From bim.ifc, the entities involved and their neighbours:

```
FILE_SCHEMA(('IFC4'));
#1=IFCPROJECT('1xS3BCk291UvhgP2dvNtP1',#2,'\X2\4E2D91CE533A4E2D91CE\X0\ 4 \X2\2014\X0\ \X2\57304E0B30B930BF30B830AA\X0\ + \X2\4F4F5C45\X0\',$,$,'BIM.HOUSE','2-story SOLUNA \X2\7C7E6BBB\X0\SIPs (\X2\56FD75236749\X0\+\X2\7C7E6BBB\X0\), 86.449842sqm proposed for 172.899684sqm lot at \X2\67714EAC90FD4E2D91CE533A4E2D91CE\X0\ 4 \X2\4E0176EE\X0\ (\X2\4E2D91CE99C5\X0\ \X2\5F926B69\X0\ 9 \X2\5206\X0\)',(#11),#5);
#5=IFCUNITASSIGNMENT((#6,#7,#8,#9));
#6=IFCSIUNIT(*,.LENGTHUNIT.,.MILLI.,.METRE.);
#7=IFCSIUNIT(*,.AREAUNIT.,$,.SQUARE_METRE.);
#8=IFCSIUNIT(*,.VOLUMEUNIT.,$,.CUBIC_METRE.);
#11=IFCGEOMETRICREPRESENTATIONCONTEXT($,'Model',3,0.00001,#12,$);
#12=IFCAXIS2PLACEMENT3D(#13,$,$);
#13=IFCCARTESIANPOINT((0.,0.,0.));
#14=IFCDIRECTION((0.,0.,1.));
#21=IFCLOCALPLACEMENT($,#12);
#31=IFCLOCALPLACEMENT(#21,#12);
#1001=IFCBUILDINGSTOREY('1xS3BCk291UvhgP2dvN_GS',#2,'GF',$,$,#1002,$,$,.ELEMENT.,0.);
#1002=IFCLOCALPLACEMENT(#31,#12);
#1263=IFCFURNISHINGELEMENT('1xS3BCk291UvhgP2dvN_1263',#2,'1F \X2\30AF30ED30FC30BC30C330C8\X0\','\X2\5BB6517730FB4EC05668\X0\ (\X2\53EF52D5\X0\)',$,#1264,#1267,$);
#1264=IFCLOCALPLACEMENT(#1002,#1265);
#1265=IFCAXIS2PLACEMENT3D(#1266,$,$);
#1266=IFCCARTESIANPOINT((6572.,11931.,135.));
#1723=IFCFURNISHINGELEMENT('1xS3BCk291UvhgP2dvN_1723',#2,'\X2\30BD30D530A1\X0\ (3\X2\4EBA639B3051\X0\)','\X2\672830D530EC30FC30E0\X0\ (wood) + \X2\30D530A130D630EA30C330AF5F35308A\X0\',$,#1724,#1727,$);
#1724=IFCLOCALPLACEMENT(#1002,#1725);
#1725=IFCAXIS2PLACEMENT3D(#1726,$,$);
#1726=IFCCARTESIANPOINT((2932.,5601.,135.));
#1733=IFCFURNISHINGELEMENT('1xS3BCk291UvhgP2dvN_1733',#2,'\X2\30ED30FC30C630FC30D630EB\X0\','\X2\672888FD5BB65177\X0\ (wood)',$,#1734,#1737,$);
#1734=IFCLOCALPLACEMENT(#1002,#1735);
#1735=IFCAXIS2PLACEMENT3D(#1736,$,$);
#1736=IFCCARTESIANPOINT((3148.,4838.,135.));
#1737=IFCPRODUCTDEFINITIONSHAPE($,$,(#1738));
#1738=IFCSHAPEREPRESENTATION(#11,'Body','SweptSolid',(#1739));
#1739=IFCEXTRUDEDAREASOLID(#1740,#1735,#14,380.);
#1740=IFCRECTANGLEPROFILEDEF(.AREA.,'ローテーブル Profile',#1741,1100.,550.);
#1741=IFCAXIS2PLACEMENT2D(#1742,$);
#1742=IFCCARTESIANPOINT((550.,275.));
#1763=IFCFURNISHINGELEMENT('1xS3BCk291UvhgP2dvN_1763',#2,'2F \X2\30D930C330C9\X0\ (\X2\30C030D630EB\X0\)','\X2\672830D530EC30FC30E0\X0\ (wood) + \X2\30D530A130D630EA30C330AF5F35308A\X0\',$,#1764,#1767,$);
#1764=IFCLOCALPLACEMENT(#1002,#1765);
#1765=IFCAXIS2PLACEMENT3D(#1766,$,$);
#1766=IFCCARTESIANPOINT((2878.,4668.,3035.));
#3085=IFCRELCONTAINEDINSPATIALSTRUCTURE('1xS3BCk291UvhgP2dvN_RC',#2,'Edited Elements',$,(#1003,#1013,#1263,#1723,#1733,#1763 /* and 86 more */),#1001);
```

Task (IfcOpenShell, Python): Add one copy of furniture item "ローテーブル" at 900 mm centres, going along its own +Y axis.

```python
import ifcopenshell
import ifcopenshell.api.geometry
import ifcopenshell.api.root
import ifcopenshell.util.element
import ifcopenshell.util.placement
import ifcopenshell.util.unit

model = ifcopenshell.open("bim.ifc")
unit_scale = ifcopenshell.util.unit.calculate_unit_scale(model)


def reuse_history(source, copy):
    """copy_class also copies each property set's owner history, people and application; keep the originals."""
    for rel in copy.IsDefinedBy:
        if rel.is_a("IfcRelDefinesByProperties") and (history := rel.RelatingPropertyDefinition.OwnerHistory):
            rel.RelatingPropertyDefinition.OwnerHistory = source.OwnerHistory
            ifcopenshell.util.element.remove_deep2(model, history)


source = model.by_guid("1xS3BCk291UvhgP2dvN_1733")
base = ifcopenshell.util.placement.get_local_placement(source.ObjectPlacement)
step = base[:3, 1] * 0.9 / unit_scale

for i in range(1, 2):
    copy = ifcopenshell.api.root.copy_class(model, product=source)
    copy.Representation = ifcopenshell.util.element.copy_deep(
        model, source.Representation, exclude=["IfcGeometricRepresentationContext", "IfcRepresentationMap"]
    )
    reuse_history(source, copy)
    matrix = base.copy()
    matrix[:3, 3] += i * step
    print("added at", matrix[:3, 3].round(3) + 0.0)
    ifcopenshell.api.geometry.edit_object_placement(model, product=copy, matrix=matrix, is_si=False)

model.write("bim_rev.ifc")
```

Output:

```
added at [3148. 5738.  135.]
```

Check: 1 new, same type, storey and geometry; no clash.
